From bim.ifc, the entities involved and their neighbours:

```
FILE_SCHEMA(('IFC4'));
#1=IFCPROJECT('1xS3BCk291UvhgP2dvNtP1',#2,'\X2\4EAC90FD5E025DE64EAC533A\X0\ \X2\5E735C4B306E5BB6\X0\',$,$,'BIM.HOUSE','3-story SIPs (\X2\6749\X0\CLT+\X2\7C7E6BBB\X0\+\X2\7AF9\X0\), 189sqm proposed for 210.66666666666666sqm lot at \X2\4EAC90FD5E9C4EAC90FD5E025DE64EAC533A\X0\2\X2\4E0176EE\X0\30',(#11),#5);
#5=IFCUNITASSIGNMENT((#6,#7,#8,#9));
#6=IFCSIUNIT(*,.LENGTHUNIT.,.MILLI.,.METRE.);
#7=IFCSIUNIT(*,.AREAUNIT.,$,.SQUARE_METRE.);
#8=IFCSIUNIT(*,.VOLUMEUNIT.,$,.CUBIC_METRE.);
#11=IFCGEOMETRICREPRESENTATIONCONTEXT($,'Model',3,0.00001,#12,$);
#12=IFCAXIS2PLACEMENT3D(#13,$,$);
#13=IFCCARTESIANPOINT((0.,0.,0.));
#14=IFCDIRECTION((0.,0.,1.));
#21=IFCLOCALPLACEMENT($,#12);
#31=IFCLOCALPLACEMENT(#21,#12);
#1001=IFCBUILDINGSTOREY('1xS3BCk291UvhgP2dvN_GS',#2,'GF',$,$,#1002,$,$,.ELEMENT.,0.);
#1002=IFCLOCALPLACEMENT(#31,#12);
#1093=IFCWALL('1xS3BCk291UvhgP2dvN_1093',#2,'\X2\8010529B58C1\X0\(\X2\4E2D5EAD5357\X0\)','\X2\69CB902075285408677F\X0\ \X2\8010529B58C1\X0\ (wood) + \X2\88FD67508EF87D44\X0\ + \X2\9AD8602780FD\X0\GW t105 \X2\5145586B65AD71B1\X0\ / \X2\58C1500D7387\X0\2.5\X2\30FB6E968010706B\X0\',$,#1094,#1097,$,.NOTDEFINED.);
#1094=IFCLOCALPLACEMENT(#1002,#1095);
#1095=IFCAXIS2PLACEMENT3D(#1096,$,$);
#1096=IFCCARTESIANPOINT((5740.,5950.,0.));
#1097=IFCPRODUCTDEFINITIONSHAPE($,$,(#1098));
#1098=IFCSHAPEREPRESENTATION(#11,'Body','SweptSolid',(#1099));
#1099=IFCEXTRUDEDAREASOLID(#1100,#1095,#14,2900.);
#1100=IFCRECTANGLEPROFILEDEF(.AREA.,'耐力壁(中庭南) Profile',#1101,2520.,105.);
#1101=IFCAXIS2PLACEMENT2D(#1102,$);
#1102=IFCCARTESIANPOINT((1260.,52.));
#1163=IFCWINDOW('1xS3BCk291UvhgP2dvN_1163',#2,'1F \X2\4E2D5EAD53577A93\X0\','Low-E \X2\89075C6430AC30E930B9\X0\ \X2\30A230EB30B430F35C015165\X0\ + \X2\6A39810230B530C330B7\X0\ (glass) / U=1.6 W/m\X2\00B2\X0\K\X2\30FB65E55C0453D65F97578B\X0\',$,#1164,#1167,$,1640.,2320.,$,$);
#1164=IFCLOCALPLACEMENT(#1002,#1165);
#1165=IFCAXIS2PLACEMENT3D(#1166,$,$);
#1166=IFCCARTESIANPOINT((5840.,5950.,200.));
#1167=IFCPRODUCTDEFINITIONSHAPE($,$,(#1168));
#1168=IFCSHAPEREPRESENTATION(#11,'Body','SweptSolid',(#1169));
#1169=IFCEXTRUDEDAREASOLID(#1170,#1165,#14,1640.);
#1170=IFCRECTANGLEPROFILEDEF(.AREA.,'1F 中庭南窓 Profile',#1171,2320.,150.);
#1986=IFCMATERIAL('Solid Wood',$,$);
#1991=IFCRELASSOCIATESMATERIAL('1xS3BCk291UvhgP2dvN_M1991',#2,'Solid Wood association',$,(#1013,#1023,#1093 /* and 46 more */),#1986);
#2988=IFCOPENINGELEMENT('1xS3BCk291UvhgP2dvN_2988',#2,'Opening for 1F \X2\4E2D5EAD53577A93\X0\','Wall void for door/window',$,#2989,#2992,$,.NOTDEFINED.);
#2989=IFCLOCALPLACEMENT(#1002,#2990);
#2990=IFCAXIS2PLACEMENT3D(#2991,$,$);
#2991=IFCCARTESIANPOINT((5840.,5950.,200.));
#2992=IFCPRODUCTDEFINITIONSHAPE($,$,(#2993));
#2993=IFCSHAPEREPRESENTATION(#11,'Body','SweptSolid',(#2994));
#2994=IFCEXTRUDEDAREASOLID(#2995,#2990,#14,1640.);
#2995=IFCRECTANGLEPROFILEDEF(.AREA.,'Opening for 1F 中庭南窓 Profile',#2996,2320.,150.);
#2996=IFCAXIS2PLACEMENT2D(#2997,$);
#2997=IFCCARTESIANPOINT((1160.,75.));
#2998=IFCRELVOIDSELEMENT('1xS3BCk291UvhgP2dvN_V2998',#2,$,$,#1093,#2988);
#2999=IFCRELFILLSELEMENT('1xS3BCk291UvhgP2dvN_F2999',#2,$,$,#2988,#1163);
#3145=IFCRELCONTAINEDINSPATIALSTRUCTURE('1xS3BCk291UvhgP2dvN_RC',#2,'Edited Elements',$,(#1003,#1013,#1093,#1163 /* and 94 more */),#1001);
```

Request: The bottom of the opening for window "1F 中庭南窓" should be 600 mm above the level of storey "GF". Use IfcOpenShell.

```python
import numpy as np
import ifcopenshell
import ifcopenshell.api.geometry
import ifcopenshell.geom
import ifcopenshell.util.element
import ifcopenshell.util.placement
import ifcopenshell.util.shape
import ifcopenshell.util.unit

model = ifcopenshell.open("bim.ifc")
unit_scale = ifcopenshell.util.unit.calculate_unit_scale(model)

window = model.by_guid("1xS3BCk291UvhgP2dvN_1163")
opening = window.FillsVoids[0].RelatingOpeningElement
storey = ifcopenshell.util.element.get_container(window, ifc_class="IfcBuildingStorey")
level = ifcopenshell.util.placement.get_local_placement(storey.ObjectPlacement)[2, 3]

# The opening's origin need not be at the sill, so measure its lowest point.
shape = ifcopenshell.geom.create_shape(ifcopenshell.geom.settings(), opening)
bottom = ifcopenshell.util.shape.get_shape_bottom_elevation(shape, shape.geometry) / unit_scale
dz = level + 0.6 / unit_scale - bottom

shift = np.array([0.0, 0.0, dz])
# The window is not placed relative to its opening, so move both.
for product in (opening, window):
    matrix = ifcopenshell.util.placement.get_local_placement(product.ObjectPlacement)
    matrix[:3, 3] += shift
    ifcopenshell.api.geometry.edit_object_placement(model, product=product, matrix=matrix, is_si=False)

print(f"moved by {dz * unit_scale:+.3f} m")

model.write("bim-out.ifc")
```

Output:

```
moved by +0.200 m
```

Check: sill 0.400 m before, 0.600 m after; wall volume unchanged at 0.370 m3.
